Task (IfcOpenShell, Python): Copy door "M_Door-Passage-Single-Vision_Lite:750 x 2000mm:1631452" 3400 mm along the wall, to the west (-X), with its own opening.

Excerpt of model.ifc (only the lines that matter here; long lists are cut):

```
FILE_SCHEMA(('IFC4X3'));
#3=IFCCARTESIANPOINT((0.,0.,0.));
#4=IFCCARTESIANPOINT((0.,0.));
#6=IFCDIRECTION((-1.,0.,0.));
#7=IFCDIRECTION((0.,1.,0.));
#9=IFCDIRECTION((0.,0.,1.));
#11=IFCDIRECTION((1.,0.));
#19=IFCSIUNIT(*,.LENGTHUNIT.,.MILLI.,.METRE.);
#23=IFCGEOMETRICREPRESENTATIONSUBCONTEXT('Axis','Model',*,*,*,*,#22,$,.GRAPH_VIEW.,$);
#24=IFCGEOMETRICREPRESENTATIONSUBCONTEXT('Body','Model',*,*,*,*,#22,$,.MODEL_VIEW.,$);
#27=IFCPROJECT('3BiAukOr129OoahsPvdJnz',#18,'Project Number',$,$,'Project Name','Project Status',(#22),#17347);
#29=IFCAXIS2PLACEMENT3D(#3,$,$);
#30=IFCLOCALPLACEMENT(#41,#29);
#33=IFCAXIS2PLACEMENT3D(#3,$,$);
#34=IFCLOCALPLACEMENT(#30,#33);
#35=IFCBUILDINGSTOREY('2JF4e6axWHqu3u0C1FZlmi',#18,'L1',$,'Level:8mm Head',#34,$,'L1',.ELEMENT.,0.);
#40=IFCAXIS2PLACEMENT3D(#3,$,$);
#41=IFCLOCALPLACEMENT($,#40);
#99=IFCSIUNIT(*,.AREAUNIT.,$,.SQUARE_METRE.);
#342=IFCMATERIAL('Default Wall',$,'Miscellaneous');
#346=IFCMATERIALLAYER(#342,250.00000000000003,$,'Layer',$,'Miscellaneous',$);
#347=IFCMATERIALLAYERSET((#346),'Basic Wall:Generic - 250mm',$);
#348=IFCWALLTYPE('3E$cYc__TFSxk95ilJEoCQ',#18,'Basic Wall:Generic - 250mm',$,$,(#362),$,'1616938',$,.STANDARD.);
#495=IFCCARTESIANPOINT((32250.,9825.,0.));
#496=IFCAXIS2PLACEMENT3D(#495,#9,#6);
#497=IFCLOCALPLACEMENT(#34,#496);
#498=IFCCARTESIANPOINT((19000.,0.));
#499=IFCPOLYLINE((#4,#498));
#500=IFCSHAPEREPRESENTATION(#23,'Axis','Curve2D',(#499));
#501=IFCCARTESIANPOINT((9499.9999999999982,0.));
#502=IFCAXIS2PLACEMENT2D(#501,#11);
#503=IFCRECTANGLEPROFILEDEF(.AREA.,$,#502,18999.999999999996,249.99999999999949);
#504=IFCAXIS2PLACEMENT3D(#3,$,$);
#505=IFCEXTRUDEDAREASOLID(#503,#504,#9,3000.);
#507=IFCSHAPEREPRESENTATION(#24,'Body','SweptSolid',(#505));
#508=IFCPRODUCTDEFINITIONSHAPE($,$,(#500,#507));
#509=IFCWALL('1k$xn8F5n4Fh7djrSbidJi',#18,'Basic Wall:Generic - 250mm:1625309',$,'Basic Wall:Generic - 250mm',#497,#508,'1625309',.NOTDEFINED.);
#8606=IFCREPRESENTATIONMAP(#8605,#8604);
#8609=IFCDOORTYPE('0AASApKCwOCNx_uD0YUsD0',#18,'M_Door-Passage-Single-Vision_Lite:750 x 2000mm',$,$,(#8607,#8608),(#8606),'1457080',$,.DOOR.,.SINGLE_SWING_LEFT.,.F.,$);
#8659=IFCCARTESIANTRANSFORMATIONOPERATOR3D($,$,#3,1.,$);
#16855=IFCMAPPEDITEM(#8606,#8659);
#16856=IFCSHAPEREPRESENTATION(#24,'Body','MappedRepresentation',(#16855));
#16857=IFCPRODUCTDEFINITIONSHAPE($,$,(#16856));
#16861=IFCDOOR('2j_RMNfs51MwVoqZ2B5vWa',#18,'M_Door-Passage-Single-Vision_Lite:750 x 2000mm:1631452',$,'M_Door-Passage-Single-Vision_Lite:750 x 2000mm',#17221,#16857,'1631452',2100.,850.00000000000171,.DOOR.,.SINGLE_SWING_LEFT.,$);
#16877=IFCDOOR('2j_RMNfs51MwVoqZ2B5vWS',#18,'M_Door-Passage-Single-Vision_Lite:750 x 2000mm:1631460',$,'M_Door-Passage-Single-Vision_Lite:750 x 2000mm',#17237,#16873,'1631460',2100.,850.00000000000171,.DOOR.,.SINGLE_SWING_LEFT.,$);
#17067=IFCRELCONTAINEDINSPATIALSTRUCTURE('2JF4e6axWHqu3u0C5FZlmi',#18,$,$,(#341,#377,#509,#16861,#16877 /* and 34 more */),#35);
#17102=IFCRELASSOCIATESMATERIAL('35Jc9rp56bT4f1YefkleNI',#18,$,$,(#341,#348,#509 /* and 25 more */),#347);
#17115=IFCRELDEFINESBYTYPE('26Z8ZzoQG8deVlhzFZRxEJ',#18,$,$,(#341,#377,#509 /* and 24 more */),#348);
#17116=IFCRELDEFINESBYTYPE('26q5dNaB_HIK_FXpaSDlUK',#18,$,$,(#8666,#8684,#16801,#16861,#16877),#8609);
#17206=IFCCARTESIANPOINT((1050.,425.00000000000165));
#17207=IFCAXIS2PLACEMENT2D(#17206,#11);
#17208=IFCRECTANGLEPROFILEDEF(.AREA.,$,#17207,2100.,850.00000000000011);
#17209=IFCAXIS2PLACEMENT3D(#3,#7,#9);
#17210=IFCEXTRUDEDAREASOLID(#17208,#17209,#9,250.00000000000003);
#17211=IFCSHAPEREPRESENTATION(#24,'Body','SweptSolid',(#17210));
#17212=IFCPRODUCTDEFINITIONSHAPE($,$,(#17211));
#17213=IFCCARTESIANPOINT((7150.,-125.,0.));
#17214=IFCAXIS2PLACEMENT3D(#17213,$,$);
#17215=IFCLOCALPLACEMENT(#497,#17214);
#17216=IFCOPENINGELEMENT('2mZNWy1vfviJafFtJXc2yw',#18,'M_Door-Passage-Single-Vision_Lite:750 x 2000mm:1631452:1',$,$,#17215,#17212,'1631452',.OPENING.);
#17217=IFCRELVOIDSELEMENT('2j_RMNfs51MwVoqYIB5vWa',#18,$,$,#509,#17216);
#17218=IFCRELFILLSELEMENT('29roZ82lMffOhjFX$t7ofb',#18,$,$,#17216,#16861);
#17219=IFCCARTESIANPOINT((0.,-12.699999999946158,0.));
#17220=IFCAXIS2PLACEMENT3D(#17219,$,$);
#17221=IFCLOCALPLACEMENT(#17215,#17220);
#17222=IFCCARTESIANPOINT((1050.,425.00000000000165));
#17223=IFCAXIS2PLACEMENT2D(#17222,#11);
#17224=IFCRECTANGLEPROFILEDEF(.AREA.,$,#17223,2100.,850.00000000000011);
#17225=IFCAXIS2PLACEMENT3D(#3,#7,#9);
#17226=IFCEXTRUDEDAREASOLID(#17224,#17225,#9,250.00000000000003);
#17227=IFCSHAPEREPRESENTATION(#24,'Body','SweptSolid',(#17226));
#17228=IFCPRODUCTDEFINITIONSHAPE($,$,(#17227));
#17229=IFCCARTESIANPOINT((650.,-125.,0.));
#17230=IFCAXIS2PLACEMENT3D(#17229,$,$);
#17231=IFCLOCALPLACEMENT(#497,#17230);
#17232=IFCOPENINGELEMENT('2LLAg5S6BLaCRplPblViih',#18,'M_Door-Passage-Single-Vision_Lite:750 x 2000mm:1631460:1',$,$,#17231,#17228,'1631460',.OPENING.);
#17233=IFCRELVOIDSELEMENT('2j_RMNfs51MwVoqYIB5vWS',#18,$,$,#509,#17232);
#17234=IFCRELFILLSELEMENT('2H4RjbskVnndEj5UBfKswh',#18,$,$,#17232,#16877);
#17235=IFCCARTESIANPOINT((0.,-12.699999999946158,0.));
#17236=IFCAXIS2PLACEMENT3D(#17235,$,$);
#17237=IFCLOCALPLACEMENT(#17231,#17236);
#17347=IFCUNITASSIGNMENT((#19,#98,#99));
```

```python
import ifcopenshell
import ifcopenshell.api.feature
import ifcopenshell.api.geometry
import ifcopenshell.api.root
import ifcopenshell.geom
import ifcopenshell.util.element
import ifcopenshell.util.placement
import ifcopenshell.util.shape

model = ifcopenshell.open("model.ifc")
settings = ifcopenshell.geom.settings()


def volume(element):
    """Net volume in cubic metres, openings subtracted."""
    shape = ifcopenshell.geom.create_shape(settings, element)
    return ifcopenshell.util.shape.get_volume(shape.geometry)


def reuse_history(source, copy):
    """copy_class also copies each property set's owner history, people and application; keep the originals."""
    for rel in copy.IsDefinedBy:
        if rel.is_a("IfcRelDefinesByProperties") and (history := rel.RelatingPropertyDefinition.OwnerHistory):
            rel.RelatingPropertyDefinition.OwnerHistory = source.OwnerHistory
            ifcopenshell.util.element.remove_deep2(model, history)


door = model.by_guid("2j_RMNfs51MwVoqZ2B5vWa")
opening = door.FillsVoids[0].RelatingOpeningElement
wall = opening.VoidsElements[0].RelatingBuildingElement
before = volume(wall)
shift = ifcopenshell.util.placement.get_local_placement(wall.ObjectPlacement)[:3, 0] * 3400.0

# copy_class copies the void relationship, type, container and properties, but no geometry.
new_opening = ifcopenshell.api.root.copy_class(model, product=opening)
new_opening.Representation = ifcopenshell.util.element.copy_deep(
    model, opening.Representation, exclude=["IfcGeometricRepresentationContext", "IfcRepresentationMap"]
)
new_opening.Name = "M_Door-Passage-Single-Vision_Lite:750 x 2000mm"
new_opening.Tag = None
new_door = ifcopenshell.api.root.copy_class(model, product=door)
new_door.Representation = ifcopenshell.util.element.copy_deep(
    model, door.Representation, exclude=["IfcGeometricRepresentationContext", "IfcRepresentationMap"]
)
new_door.Name = "M_Door-Passage-Single-Vision_Lite:750 x 2000mm"
new_door.Tag = None
reuse_history(door, new_door)
ifcopenshell.api.feature.add_filling(model, opening=new_opening, element=new_door)

for old, new in ((opening, new_opening), (door, new_door)):
    matrix = ifcopenshell.util.placement.get_local_placement(old.ObjectPlacement)
    matrix[:3, 3] += shift
    ifcopenshell.api.geometry.edit_object_placement(model, product=new, matrix=matrix, is_si=False)

after = volume(wall)

print(f"wall volume {before:.3f} -> {after:.3f} m3")

model.write("model-out.ifc")
```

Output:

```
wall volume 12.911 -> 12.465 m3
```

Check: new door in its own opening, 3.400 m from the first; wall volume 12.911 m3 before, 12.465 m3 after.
